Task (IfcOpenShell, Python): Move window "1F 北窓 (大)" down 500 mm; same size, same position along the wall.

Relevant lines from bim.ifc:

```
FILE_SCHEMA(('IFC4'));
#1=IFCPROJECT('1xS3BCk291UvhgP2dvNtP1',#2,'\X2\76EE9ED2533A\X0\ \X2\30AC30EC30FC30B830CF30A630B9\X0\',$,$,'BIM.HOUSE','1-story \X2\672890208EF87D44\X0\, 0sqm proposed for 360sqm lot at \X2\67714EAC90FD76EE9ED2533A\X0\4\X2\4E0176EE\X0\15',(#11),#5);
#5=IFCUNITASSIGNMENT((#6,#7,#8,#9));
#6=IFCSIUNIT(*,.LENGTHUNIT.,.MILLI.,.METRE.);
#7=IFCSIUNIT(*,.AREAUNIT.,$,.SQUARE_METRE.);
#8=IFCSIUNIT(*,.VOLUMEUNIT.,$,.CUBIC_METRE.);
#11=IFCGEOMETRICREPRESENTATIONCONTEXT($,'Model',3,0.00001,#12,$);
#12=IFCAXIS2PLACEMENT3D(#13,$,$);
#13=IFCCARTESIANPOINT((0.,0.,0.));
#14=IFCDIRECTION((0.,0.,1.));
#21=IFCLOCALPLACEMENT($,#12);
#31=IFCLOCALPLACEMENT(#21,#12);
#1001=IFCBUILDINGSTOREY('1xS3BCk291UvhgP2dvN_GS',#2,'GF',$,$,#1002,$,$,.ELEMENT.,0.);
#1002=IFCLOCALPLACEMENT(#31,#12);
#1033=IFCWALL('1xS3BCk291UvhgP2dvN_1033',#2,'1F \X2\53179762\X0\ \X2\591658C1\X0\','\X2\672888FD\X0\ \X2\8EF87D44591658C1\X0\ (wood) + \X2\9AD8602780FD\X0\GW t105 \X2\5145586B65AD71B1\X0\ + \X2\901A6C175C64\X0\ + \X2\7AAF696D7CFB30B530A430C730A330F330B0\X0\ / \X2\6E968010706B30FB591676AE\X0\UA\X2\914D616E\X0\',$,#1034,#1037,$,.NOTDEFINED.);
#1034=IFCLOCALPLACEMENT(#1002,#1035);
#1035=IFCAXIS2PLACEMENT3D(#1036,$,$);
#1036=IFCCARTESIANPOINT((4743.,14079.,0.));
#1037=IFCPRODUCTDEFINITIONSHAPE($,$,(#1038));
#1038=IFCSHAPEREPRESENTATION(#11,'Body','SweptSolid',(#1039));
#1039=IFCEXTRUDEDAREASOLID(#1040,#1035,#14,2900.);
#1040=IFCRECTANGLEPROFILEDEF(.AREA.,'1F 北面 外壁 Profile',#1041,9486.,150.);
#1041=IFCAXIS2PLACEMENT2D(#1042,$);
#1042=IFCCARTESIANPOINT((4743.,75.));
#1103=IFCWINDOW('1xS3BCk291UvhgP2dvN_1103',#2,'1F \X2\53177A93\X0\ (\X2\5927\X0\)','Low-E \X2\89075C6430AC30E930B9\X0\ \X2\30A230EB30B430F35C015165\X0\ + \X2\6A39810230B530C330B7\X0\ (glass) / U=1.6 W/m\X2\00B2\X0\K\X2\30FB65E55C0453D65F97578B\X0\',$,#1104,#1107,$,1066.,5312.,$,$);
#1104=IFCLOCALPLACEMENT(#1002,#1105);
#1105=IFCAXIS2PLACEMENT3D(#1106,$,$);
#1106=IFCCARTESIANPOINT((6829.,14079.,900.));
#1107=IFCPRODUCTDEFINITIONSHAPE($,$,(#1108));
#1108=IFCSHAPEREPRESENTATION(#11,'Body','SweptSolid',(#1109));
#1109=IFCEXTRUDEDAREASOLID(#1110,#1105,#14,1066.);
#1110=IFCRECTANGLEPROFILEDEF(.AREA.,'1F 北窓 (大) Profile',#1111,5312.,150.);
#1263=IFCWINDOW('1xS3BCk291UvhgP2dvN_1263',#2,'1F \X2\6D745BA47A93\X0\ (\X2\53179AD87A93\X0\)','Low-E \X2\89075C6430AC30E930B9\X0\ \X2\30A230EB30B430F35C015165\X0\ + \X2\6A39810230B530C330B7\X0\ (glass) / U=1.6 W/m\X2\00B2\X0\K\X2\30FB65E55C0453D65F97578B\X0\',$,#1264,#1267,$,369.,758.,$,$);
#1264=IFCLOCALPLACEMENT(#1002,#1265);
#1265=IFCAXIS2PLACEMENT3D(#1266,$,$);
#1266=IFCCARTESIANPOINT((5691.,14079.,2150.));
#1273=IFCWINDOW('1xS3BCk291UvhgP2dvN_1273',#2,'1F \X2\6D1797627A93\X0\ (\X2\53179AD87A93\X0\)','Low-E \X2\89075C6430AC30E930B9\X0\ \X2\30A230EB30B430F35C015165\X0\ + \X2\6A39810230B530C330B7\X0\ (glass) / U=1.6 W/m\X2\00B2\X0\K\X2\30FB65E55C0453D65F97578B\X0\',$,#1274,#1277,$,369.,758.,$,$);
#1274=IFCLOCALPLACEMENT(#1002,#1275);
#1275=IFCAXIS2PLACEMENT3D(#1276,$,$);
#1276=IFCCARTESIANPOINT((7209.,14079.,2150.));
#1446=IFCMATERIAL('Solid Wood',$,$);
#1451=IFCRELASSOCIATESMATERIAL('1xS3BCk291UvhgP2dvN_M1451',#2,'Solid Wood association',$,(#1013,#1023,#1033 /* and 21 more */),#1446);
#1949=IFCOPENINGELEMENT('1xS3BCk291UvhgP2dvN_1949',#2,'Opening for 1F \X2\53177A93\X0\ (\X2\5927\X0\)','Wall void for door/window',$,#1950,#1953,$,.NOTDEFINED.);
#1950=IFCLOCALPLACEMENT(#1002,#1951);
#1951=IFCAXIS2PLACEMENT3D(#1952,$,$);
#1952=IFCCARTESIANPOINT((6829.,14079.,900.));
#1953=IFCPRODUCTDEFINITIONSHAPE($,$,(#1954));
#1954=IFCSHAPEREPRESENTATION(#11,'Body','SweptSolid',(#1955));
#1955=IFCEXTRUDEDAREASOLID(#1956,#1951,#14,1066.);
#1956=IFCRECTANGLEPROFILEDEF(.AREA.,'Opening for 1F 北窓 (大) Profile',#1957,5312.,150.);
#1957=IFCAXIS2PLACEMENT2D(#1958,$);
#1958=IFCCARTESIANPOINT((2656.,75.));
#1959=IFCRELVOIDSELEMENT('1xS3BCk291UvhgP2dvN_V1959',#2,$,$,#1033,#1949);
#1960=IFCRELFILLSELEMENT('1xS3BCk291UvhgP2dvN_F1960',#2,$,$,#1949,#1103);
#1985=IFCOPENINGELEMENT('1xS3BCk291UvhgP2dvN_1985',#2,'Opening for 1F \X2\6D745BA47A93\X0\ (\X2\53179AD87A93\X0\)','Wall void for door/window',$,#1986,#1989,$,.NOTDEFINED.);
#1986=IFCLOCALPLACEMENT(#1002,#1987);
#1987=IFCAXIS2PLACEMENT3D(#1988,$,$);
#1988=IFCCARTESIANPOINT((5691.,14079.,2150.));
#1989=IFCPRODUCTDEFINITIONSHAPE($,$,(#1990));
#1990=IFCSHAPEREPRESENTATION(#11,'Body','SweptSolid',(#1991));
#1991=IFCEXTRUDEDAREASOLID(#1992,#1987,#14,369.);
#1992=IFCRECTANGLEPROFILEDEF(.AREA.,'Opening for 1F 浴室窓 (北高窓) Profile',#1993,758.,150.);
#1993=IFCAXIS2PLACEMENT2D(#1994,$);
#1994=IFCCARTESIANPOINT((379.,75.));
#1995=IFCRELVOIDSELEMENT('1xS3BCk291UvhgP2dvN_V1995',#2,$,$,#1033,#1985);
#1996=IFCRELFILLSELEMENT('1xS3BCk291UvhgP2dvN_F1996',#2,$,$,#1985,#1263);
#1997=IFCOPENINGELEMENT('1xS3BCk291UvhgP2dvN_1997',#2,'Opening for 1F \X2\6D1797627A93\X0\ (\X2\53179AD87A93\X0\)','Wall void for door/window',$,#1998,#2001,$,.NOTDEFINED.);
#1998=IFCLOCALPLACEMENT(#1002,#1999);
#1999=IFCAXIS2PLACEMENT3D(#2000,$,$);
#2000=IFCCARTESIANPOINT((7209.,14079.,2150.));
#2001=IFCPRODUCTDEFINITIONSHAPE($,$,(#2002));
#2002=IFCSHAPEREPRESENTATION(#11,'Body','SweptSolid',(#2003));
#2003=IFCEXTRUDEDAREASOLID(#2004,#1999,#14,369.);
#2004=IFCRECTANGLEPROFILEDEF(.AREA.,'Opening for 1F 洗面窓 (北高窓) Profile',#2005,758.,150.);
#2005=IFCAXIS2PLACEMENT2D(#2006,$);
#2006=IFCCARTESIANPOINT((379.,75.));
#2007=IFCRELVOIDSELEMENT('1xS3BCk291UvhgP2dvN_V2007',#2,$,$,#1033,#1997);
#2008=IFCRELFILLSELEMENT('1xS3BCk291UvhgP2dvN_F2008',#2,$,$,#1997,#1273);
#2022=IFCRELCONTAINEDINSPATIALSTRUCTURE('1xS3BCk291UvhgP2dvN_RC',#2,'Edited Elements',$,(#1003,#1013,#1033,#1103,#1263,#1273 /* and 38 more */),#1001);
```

```python
import numpy as np
import ifcopenshell
import ifcopenshell.api.geometry
import ifcopenshell.util.placement
import ifcopenshell.util.unit

model = ifcopenshell.open("bim.ifc")
unit_scale = ifcopenshell.util.unit.calculate_unit_scale(model)

window = model.by_id(1103)
opening = window.FillsVoids[0].RelatingOpeningElement
dz = -0.5 / unit_scale

shift = np.array([0.0, 0.0, dz])
# The window is not placed relative to its opening, so move both.
for product in (opening, window):
    matrix = ifcopenshell.util.placement.get_local_placement(product.ObjectPlacement)
    matrix[:3, 3] += shift
    ifcopenshell.api.geometry.edit_object_placement(model, product=product, matrix=matrix, is_si=False)

print(f"moved by {dz * unit_scale:+.3f} m")

model.write("bim_edited.ifc")
```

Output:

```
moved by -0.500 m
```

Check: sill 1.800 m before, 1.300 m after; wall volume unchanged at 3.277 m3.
